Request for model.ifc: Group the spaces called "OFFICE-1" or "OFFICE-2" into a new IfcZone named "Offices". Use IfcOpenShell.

First a look at what the model holds.

```python
import ifcopenshell

model = ifcopenshell.open("model.ifc")
print(model.schema)
seen = {}
for space in model.by_type("IfcSpace"):
    seen[space.Name] = seen.get(space.Name, 0) + 1
for name, count in sorted(seen.items(), key=str):
    print(count, "x", name)
print("zones:", [z.Name for z in model.by_type("IfcZone")][:20])
```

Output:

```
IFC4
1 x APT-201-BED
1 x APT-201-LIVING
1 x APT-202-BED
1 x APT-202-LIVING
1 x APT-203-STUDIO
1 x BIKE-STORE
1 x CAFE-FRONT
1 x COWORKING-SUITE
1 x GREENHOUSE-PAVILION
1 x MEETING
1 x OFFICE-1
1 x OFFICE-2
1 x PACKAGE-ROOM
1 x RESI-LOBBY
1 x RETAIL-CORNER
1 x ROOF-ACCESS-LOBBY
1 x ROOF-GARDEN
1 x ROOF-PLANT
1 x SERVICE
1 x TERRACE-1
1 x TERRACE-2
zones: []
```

```python
import ifcopenshell
import ifcopenshell.api.group
import ifcopenshell.api.root

model = ifcopenshell.open("model.ifc")

names = {"OFFICE-1", "OFFICE-2"}
spaces = [s for s in model.by_type("IfcSpace") if s.Name in names]

zone = ifcopenshell.api.root.create_entity(model, ifc_class="IfcZone", name="Offices")
ifcopenshell.api.group.assign_group(model, products=spaces, group=zone)
print(len(spaces), "spaces in", zone.Name)

model.write("model_rev.ifc")
```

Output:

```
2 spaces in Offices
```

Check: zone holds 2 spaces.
